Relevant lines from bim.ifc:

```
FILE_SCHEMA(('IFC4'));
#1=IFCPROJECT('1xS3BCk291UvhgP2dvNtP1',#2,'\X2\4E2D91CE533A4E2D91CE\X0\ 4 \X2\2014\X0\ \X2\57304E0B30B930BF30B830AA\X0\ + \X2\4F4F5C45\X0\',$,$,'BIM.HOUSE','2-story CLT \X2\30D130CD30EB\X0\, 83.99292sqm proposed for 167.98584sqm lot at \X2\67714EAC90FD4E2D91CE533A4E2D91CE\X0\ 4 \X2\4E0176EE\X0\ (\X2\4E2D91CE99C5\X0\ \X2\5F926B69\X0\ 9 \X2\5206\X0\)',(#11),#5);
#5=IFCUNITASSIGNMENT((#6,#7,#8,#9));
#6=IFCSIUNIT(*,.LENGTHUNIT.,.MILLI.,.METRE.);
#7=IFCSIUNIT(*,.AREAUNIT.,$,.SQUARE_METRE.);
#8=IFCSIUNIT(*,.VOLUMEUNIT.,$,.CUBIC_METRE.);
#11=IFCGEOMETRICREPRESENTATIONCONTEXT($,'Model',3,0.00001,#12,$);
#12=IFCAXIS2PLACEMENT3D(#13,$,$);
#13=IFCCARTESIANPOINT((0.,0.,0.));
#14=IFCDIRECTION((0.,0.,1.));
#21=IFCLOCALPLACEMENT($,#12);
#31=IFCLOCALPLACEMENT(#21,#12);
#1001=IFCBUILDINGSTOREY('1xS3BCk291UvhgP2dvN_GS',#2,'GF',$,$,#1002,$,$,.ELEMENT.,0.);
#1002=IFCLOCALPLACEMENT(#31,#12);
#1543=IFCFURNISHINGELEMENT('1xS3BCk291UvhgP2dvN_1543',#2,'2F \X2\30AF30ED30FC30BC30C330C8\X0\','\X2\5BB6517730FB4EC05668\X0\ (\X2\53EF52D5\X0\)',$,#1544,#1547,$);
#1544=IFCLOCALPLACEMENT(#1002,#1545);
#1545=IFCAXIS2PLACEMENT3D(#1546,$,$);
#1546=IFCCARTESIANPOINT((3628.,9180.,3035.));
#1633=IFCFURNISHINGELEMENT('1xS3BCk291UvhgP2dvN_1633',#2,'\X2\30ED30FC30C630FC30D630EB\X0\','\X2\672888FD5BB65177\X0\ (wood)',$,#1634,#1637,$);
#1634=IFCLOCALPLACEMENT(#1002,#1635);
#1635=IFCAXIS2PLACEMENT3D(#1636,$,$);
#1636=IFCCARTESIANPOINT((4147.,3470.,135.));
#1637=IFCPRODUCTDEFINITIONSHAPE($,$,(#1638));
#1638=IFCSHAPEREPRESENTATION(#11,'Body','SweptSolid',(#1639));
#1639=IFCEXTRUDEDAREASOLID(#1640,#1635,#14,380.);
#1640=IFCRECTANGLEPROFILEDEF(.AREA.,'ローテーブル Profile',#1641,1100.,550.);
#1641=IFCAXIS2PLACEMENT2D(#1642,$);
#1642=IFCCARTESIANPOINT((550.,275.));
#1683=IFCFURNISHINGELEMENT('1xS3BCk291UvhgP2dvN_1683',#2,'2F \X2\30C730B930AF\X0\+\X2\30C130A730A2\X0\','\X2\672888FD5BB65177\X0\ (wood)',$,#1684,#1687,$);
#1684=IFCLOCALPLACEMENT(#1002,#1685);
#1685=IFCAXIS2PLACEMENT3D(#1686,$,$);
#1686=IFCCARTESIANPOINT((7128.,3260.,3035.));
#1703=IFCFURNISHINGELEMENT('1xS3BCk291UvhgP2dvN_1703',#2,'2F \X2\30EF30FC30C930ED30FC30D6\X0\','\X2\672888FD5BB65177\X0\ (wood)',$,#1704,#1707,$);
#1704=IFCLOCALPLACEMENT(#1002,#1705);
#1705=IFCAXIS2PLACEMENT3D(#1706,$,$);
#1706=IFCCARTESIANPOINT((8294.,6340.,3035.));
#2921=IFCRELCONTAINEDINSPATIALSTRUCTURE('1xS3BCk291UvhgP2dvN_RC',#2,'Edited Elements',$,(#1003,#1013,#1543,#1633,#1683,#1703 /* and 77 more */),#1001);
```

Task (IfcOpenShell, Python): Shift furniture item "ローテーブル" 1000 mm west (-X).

```python
import ifcopenshell
import ifcopenshell.api.geometry
import ifcopenshell.util.placement

model = ifcopenshell.open("bim.ifc")

item = model.by_guid("1xS3BCk291UvhgP2dvN_1633")
matrix = ifcopenshell.util.placement.get_local_placement(item.ObjectPlacement)
matrix[0, 3] -= 1000.0
ifcopenshell.api.geometry.edit_object_placement(model, product=item, matrix=matrix, is_si=False)

print(ifcopenshell.util.placement.get_local_placement(item.ObjectPlacement).round(3) + 0.0)

model.write("bim_updated.ifc")
```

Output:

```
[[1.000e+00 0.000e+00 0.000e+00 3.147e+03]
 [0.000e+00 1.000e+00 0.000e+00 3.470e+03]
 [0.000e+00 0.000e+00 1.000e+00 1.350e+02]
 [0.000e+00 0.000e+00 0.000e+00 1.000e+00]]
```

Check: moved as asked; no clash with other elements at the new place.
